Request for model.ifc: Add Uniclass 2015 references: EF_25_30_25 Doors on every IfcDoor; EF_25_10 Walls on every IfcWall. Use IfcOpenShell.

First a look at what the model holds.

```python
import ifcopenshell

model = ifcopenshell.open("model.ifc")
print(model.schema)
print("classifications:", [c.Name for c in model.by_type("IfcClassification")])
for ifc_class in ("IfcDoor", "IfcRoof", "IfcStair", "IfcWall", "IfcWindow"):
    print(ifc_class, len(model.by_type(ifc_class)))
```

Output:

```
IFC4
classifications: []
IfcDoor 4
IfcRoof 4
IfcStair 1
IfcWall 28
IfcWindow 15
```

```python
import ifcopenshell
import ifcopenshell.api.classification

model = ifcopenshell.open("model.ifc")

system = ifcopenshell.api.classification.add_classification(model, classification="Uniclass 2015")

codes = {
    "IfcDoor": ("EF_25_30_25", "Doors"),
    "IfcWall": ("EF_25_10", "Walls"),
}
for ifc_class, (code, name) in codes.items():
    products = model.by_type(ifc_class)
    ifcopenshell.api.classification.add_reference(
        model, products=products, classification=system, identification=code, name=name
    )
    print(code, len(products))

model.write("model_edited.ifc")
```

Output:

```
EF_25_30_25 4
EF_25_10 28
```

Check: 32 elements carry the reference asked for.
